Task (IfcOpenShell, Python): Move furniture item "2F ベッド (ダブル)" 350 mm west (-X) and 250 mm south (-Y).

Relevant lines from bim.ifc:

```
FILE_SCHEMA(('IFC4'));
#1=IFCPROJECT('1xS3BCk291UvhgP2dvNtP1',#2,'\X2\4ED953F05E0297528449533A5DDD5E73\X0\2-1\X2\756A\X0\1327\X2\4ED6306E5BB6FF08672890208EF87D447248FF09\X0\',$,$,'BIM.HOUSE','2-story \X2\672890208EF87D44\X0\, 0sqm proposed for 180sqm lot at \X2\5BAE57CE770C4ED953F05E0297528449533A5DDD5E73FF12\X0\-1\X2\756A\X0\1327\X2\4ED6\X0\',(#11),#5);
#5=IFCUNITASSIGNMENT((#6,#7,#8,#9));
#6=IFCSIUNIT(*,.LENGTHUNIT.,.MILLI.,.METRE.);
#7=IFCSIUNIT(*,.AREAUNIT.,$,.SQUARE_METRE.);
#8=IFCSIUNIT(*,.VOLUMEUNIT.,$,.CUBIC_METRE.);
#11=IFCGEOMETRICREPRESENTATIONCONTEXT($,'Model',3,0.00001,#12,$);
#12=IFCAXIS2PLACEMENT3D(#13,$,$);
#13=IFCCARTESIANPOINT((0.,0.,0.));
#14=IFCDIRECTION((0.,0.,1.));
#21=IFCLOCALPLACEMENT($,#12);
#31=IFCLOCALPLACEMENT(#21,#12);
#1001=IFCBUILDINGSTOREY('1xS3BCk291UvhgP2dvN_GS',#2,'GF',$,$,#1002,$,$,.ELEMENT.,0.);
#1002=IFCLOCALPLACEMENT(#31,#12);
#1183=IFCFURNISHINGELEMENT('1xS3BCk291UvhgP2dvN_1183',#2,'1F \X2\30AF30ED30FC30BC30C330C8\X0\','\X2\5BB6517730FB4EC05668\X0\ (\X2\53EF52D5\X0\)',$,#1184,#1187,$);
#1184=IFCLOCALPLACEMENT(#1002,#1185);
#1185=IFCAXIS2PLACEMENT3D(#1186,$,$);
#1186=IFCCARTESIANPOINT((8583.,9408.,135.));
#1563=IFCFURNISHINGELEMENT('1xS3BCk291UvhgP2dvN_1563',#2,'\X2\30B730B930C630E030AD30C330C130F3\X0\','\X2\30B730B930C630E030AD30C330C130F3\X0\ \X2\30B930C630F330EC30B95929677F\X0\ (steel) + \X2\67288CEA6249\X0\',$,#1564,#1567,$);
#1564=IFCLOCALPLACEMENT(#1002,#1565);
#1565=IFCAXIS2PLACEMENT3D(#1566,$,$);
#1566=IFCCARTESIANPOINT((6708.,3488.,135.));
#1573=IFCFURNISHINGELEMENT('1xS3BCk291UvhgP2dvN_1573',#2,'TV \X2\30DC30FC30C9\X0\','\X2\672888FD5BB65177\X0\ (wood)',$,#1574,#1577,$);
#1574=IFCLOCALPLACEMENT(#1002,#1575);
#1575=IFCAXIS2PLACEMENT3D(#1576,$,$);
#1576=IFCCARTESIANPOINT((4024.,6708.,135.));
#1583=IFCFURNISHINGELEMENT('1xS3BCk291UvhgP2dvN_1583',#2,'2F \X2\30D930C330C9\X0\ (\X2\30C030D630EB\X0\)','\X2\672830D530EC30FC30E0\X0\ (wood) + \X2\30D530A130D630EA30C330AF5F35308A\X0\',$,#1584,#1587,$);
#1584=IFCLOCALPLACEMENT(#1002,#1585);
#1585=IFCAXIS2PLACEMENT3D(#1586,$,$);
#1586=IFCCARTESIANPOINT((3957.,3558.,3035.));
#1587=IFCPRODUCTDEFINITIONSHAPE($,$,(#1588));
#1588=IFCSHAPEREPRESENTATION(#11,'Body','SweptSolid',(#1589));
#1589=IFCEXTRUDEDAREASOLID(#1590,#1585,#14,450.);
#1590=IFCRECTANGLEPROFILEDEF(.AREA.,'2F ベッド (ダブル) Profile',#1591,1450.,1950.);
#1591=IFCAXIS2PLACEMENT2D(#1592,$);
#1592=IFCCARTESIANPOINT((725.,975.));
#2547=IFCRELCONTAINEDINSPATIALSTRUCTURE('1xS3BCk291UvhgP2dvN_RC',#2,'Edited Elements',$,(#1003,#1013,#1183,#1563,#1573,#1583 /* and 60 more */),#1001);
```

```python
import ifcopenshell
import ifcopenshell.api.geometry
import ifcopenshell.util.placement

model = ifcopenshell.open("bim.ifc")

item = model.by_id(1583)
matrix = ifcopenshell.util.placement.get_local_placement(item.ObjectPlacement)
matrix[0, 3] -= 350.0
matrix[1, 3] -= 250.0
ifcopenshell.api.geometry.edit_object_placement(model, product=item, matrix=matrix, is_si=False)

print(ifcopenshell.util.placement.get_local_placement(item.ObjectPlacement).round(3) + 0.0)

model.write("bim_updated.ifc")
```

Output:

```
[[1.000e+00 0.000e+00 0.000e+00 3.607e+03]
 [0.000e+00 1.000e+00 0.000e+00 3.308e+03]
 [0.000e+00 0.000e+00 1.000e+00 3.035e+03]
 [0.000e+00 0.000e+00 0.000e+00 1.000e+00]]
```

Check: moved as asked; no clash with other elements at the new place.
